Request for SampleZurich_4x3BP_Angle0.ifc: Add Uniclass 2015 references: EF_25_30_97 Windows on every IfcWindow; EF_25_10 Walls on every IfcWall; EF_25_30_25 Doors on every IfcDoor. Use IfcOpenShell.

First a look at what the model holds.

```python
import ifcopenshell

model = ifcopenshell.open("SampleZurich_4x3BP_Angle0.ifc")
print(model.schema)
print("classifications:", [c.Name for c in model.by_type("IfcClassification")])
for ifc_class in ("IfcDoor", "IfcRoof", "IfcStair", "IfcWall", "IfcWindow"):
    print(ifc_class, len(model.by_type(ifc_class)))
```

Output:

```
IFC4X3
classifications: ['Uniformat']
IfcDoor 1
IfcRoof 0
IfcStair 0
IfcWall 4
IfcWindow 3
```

```python
import ifcopenshell
import ifcopenshell.api.classification

model = ifcopenshell.open("SampleZurich_4x3BP_Angle0.ifc")

system = ifcopenshell.api.classification.add_classification(model, classification="Uniclass 2015")

codes = {
    "IfcWindow": ("EF_25_30_97", "Windows"),
    "IfcWall": ("EF_25_10", "Walls"),
    "IfcDoor": ("EF_25_30_25", "Doors"),
}
for ifc_class, (code, name) in codes.items():
    products = model.by_type(ifc_class)
    ifcopenshell.api.classification.add_reference(
        model, products=products, classification=system, identification=code, name=name
    )
    print(code, len(products))

model.write("SampleZurich_4x3BP_Angle0_edited.ifc")
```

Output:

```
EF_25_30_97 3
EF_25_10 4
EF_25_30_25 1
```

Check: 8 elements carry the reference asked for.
